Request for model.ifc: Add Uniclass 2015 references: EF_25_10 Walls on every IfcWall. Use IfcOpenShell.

First a look at what the model holds.

```python
import ifcopenshell

model = ifcopenshell.open("model.ifc")
print(model.schema)
print("classifications:", [c.Name for c in model.by_type("IfcClassification")])
for ifc_class in ("IfcDoor", "IfcRoof", "IfcStair", "IfcWall", "IfcWindow"):
    print(ifc_class, len(model.by_type(ifc_class)))
```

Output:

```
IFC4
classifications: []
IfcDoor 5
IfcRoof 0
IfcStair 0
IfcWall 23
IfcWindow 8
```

```python
import ifcopenshell
import ifcopenshell.api.classification

model = ifcopenshell.open("model.ifc")

system = ifcopenshell.api.classification.add_classification(model, classification="Uniclass 2015")

codes = {
    "IfcWall": ("EF_25_10", "Walls"),
}
for ifc_class, (code, name) in codes.items():
    products = model.by_type(ifc_class)
    ifcopenshell.api.classification.add_reference(
        model, products=products, classification=system, identification=code, name=name
    )
    print(code, len(products))

model.write("model_edited.ifc")
```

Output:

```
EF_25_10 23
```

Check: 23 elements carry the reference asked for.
